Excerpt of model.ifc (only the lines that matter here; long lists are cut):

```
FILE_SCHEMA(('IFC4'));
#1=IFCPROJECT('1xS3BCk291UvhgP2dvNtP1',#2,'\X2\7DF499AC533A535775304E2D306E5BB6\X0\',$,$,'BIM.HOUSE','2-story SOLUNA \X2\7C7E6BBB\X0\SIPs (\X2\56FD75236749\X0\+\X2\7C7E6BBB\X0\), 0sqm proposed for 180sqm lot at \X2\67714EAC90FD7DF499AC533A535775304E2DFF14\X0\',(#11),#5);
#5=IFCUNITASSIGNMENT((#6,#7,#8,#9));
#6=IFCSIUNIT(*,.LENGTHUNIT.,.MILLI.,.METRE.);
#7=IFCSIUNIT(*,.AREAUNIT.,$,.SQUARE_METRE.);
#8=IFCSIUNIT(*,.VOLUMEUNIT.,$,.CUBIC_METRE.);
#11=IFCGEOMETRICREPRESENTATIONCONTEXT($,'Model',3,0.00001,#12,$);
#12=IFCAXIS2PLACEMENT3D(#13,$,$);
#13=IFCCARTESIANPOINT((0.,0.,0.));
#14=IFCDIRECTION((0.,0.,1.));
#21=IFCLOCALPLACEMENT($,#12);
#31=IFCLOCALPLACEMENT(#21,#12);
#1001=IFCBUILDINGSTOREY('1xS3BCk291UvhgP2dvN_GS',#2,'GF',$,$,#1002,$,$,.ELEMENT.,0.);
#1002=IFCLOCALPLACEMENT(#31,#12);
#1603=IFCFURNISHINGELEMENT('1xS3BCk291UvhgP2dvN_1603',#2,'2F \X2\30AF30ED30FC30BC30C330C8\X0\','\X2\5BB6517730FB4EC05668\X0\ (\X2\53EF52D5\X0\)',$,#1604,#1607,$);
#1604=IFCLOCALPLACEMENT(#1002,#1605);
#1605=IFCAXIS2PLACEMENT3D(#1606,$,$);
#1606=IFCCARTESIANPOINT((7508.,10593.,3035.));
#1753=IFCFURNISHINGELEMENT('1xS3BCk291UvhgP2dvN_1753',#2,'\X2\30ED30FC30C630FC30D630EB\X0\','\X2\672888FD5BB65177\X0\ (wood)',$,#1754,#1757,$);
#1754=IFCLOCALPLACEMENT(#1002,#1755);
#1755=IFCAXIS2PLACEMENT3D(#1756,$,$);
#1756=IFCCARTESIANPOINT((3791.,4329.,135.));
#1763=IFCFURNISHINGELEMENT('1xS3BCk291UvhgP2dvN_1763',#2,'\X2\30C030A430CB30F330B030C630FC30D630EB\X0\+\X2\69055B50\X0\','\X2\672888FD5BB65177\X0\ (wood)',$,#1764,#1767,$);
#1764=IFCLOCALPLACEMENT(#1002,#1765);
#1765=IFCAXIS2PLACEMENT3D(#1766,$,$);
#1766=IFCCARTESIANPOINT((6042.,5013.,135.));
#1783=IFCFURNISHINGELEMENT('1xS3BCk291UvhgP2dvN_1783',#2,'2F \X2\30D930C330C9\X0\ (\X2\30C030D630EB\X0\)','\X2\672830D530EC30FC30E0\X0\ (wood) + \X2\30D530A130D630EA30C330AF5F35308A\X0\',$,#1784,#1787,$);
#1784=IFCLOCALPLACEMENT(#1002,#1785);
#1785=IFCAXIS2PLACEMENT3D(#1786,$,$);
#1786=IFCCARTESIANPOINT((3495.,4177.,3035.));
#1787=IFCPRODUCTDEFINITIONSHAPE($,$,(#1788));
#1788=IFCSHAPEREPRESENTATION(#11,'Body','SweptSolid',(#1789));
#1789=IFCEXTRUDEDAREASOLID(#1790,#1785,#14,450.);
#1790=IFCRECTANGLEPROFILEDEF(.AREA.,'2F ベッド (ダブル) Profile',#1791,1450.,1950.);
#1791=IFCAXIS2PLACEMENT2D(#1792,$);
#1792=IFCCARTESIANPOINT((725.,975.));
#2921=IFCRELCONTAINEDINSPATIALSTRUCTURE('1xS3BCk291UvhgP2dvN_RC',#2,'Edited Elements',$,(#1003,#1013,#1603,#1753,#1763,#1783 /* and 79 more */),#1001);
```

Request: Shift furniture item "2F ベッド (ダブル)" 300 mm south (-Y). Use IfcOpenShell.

```python
import ifcopenshell
import ifcopenshell.api.geometry
import ifcopenshell.util.placement

model = ifcopenshell.open("model.ifc")

item = model.by_guid("1xS3BCk291UvhgP2dvN_1783")
matrix = ifcopenshell.util.placement.get_local_placement(item.ObjectPlacement)
matrix[1, 3] -= 300.0
ifcopenshell.api.geometry.edit_object_placement(model, product=item, matrix=matrix, is_si=False)

print(ifcopenshell.util.placement.get_local_placement(item.ObjectPlacement).round(3) + 0.0)

model.write("model_rev.ifc")
```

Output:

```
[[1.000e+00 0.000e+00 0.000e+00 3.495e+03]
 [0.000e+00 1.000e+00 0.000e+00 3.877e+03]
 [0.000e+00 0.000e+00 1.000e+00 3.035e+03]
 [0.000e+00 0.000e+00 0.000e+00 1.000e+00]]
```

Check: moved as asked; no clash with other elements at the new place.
